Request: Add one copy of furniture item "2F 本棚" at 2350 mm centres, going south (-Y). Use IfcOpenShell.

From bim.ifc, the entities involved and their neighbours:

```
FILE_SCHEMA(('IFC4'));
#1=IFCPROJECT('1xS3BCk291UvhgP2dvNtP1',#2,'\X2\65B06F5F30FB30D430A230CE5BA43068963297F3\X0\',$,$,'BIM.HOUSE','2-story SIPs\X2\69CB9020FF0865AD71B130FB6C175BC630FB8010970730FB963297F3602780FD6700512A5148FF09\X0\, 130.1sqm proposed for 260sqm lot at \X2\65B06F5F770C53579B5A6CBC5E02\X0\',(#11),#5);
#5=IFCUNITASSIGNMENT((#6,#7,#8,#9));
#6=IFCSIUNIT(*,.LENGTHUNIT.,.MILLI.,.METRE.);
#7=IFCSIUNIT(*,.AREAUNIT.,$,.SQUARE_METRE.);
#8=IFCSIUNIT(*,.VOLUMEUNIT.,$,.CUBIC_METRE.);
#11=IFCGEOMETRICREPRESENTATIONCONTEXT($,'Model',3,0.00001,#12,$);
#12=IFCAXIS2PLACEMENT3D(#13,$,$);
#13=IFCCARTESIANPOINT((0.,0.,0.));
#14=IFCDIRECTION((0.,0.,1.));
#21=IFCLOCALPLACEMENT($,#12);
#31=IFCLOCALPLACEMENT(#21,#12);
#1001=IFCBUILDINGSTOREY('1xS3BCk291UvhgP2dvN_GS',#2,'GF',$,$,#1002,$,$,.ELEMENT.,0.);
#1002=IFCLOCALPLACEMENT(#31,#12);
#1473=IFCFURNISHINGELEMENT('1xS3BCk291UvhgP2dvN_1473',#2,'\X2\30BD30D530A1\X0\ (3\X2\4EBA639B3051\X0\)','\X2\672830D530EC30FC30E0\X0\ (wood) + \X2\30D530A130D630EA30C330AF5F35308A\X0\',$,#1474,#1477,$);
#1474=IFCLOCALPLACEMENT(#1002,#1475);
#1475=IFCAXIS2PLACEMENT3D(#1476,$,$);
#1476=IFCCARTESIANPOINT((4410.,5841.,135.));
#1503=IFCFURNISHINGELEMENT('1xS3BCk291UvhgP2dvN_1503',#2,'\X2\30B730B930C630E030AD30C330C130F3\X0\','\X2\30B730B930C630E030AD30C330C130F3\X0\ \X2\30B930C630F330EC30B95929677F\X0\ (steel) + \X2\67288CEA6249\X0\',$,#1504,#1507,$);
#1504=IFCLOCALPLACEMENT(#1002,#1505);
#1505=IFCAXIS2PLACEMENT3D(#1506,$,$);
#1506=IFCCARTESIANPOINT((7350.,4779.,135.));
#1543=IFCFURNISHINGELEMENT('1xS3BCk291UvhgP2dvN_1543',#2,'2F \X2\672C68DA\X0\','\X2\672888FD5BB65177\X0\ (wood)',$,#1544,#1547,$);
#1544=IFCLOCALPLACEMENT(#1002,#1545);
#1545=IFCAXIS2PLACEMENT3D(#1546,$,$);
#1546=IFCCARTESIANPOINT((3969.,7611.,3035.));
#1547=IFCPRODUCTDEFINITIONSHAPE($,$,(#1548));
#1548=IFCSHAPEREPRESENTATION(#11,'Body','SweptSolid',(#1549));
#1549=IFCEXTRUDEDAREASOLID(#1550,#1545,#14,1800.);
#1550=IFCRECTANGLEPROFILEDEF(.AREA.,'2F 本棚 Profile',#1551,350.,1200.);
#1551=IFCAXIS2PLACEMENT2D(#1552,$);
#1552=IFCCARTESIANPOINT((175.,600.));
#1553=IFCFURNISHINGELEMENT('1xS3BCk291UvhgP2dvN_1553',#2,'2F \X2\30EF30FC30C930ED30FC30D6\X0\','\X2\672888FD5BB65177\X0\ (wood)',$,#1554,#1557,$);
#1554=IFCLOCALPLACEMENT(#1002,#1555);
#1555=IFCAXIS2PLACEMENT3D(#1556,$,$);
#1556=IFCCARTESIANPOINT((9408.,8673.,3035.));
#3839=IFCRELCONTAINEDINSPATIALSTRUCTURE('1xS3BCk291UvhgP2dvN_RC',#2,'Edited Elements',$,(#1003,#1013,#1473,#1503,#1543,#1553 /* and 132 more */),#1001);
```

```python
import numpy as np
import ifcopenshell
import ifcopenshell.api.geometry
import ifcopenshell.api.root
import ifcopenshell.util.element
import ifcopenshell.util.placement
import ifcopenshell.util.unit

model = ifcopenshell.open("bim.ifc")
unit_scale = ifcopenshell.util.unit.calculate_unit_scale(model)


def reuse_history(source, copy):
    """copy_class also copies each property set's owner history, people and application; keep the originals."""
    for rel in copy.IsDefinedBy:
        if rel.is_a("IfcRelDefinesByProperties") and (history := rel.RelatingPropertyDefinition.OwnerHistory):
            rel.RelatingPropertyDefinition.OwnerHistory = source.OwnerHistory
            ifcopenshell.util.element.remove_deep2(model, history)


source = model.by_guid("1xS3BCk291UvhgP2dvN_1543")
base = ifcopenshell.util.placement.get_local_placement(source.ObjectPlacement)
step = np.array([0.0, -1.0, 0.0]) * 2.35 / unit_scale

for i in range(1, 2):
    copy = ifcopenshell.api.root.copy_class(model, product=source)
    copy.Representation = ifcopenshell.util.element.copy_deep(
        model, source.Representation, exclude=["IfcGeometricRepresentationContext", "IfcRepresentationMap"]
    )
    reuse_history(source, copy)
    matrix = base.copy()
    matrix[:3, 3] += i * step
    print("added at", matrix[:3, 3].round(3) + 0.0)
    ifcopenshell.api.geometry.edit_object_placement(model, product=copy, matrix=matrix, is_si=False)

model.write("bim_v2.ifc")
```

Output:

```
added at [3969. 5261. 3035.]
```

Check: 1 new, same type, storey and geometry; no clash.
